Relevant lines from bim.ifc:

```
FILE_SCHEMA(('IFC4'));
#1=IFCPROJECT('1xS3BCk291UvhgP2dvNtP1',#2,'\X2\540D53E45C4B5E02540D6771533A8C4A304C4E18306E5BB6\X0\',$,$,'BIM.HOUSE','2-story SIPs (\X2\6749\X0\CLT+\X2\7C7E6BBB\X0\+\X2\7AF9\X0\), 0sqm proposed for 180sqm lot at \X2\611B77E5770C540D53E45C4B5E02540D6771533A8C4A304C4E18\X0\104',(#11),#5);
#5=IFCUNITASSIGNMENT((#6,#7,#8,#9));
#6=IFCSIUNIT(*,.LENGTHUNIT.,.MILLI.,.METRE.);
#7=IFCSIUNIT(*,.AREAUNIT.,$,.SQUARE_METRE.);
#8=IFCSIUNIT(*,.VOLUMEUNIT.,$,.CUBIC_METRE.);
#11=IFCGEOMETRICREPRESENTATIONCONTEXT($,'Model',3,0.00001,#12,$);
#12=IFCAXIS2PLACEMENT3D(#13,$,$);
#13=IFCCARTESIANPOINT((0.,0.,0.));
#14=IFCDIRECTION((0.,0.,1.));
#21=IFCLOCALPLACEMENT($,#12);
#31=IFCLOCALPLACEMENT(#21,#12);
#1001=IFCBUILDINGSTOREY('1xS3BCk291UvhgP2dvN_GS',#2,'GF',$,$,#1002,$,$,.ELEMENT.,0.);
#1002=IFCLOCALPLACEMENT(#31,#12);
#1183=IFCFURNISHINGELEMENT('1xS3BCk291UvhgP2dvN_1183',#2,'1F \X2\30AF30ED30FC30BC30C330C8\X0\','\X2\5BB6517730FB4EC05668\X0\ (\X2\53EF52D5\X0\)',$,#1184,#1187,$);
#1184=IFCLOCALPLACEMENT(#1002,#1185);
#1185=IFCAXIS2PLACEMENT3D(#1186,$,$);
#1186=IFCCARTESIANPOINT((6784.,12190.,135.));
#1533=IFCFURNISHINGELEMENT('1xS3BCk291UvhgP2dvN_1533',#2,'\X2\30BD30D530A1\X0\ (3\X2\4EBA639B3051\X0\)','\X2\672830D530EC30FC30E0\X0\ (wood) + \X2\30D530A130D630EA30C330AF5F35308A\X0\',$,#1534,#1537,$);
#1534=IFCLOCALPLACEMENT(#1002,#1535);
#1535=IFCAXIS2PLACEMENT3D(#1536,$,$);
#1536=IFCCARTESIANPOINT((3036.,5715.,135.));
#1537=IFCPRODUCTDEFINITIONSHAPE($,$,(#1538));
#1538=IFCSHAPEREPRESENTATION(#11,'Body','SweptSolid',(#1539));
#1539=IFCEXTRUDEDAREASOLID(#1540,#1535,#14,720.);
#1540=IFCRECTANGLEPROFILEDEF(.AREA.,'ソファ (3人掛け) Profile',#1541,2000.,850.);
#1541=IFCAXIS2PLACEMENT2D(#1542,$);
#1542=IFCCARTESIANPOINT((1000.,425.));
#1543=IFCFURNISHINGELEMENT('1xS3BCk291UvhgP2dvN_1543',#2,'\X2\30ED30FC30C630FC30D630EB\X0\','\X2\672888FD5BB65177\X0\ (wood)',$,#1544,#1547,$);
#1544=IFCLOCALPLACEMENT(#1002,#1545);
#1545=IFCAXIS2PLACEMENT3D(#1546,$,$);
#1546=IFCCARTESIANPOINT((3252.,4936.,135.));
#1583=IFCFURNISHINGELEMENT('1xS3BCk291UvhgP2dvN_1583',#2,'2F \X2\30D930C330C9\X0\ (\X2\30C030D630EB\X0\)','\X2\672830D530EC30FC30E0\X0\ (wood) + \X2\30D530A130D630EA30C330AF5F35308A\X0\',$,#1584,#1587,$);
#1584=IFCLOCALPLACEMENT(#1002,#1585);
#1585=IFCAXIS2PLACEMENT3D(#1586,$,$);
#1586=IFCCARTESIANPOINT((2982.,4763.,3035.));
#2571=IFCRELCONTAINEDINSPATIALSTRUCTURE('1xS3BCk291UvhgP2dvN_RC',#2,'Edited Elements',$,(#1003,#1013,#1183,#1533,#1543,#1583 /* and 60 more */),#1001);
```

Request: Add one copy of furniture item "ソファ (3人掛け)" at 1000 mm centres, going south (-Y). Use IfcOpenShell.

```python
import numpy as np
import ifcopenshell
import ifcopenshell.api.geometry
import ifcopenshell.api.root
import ifcopenshell.util.element
import ifcopenshell.util.placement
import ifcopenshell.util.unit

model = ifcopenshell.open("bim.ifc")
unit_scale = ifcopenshell.util.unit.calculate_unit_scale(model)


def reuse_history(source, copy):
    """copy_class also copies each property set's owner history, people and application; keep the originals."""
    for rel in copy.IsDefinedBy:
        if rel.is_a("IfcRelDefinesByProperties") and (history := rel.RelatingPropertyDefinition.OwnerHistory):
            rel.RelatingPropertyDefinition.OwnerHistory = source.OwnerHistory
            ifcopenshell.util.element.remove_deep2(model, history)


source = model.by_guid("1xS3BCk291UvhgP2dvN_1533")
base = ifcopenshell.util.placement.get_local_placement(source.ObjectPlacement)
step = np.array([0.0, -1.0, 0.0]) * 1 / unit_scale

for i in range(1, 2):
    copy = ifcopenshell.api.root.copy_class(model, product=source)
    copy.Representation = ifcopenshell.util.element.copy_deep(
        model, source.Representation, exclude=["IfcGeometricRepresentationContext", "IfcRepresentationMap"]
    )
    reuse_history(source, copy)
    matrix = base.copy()
    matrix[:3, 3] += i * step
    print("added at", matrix[:3, 3].round(3) + 0.0)
    ifcopenshell.api.geometry.edit_object_placement(model, product=copy, matrix=matrix, is_si=False)

model.write("bim_rev.ifc")
```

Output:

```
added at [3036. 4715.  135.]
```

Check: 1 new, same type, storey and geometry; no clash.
